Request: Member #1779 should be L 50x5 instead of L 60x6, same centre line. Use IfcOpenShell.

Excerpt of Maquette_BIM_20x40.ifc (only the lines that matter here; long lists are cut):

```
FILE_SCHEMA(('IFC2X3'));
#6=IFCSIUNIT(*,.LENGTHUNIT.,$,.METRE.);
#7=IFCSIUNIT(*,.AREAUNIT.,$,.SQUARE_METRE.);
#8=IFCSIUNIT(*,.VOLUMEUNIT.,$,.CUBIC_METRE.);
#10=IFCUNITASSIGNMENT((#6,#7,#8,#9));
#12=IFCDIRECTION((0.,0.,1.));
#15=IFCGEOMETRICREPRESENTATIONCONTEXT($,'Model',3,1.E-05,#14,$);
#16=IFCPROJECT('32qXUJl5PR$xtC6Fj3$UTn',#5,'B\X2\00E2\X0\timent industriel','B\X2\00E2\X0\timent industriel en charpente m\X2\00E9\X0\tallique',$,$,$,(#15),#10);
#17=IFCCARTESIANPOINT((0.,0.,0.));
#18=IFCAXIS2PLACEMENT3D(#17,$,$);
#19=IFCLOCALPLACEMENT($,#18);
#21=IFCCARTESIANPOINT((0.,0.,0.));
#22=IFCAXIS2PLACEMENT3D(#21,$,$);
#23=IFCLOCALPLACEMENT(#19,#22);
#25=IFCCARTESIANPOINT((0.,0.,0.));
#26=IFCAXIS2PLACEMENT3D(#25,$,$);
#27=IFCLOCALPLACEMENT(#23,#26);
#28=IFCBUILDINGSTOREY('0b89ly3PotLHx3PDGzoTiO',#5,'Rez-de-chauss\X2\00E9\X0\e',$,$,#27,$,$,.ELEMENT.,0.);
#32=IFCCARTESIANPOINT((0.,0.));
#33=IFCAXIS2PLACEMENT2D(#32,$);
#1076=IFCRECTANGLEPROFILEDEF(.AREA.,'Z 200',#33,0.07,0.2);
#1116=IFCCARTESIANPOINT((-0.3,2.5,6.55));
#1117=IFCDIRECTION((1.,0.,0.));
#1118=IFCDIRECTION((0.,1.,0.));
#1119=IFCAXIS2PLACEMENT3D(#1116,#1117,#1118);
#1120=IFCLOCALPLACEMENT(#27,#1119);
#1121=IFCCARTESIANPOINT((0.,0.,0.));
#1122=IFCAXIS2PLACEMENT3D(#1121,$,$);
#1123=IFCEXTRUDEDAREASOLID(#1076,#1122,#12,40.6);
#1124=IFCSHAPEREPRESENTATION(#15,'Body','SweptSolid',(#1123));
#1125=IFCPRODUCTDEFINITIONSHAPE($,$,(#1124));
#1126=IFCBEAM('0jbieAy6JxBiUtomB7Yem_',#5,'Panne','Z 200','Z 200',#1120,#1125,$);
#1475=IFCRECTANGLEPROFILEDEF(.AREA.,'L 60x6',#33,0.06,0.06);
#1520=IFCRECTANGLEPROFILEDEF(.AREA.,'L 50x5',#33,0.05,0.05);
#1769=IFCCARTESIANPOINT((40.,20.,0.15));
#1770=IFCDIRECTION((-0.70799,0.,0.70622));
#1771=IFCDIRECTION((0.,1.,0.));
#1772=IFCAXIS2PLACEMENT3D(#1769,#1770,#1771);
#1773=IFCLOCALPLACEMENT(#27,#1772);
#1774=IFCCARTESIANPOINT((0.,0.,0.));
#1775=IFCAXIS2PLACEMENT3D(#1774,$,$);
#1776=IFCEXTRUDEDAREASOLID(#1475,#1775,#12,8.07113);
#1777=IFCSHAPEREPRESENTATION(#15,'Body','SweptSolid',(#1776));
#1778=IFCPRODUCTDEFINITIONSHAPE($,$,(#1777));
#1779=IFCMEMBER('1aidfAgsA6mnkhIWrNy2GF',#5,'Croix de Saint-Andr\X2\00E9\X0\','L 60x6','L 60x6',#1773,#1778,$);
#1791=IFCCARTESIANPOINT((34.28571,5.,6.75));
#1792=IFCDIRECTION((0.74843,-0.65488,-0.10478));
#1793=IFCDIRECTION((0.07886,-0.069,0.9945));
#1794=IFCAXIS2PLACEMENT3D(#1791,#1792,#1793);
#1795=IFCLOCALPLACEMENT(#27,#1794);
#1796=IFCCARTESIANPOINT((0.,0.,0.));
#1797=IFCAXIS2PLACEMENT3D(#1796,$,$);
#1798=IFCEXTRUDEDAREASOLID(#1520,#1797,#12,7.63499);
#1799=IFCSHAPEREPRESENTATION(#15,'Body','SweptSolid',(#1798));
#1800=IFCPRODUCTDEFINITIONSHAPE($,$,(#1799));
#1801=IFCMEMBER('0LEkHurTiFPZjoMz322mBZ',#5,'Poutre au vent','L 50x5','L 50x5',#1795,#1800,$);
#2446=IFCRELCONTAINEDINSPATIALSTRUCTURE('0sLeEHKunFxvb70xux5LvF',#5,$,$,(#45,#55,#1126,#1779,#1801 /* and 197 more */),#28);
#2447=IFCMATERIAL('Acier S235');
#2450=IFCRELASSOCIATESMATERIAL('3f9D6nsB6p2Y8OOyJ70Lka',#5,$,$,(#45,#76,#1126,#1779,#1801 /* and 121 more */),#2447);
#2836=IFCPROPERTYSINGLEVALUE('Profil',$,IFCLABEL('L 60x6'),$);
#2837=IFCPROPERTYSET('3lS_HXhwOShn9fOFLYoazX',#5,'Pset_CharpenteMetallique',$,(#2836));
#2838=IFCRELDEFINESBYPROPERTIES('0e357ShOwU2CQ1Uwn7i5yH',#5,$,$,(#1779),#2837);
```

```python
import ifcopenshell
import ifcopenshell.api.pset
import ifcopenshell.util.element

model = ifcopenshell.open("Maquette_BIM_20x40.ifc")

member = model.by_guid("1aidfAgsA6mnkhIWrNy2GF")
source = next(p for p in model.by_type("IfcRectangleProfileDef") if p.ProfileName == "L 50x5")

body = next(r for r in member.Representation.Representations if r.RepresentationIdentifier == "Body")
solid = body.Items[0]
old_profile = solid.SweptArea

# Copy the section's sizes but keep this member's own profile position.
profile = ifcopenshell.util.element.copy(model, source)
profile.Position = old_profile.Position
solid.SweptArea = profile
if not model.get_total_inverses(old_profile):
    ifcopenshell.util.element.remove_deep2(model, old_profile)
member.Description = member.Description.replace("L 60x6", "L 50x5")
member.ObjectType = member.ObjectType.replace("L 60x6", "L 50x5")
pset = model.by_id(ifcopenshell.util.element.get_pset(member, "Pset_CharpenteMetallique", should_inherit=False)["id"])
ifcopenshell.api.pset.edit_pset(model, pset=pset, properties={"Profil": "L 50x5"})

print(solid.SweptArea)

model.write("Maquette_BIM_20x40_edited.ifc")
```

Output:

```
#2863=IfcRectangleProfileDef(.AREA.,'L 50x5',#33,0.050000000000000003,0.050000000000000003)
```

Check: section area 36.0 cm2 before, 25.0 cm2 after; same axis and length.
